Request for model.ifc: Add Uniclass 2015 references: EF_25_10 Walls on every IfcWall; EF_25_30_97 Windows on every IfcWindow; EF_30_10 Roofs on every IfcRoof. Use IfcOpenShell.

First a look at what the model holds.

```python
import ifcopenshell

model = ifcopenshell.open("model.ifc")
print(model.schema)
print("classifications:", [c.Name for c in model.by_type("IfcClassification")])
for ifc_class in ("IfcDoor", "IfcRoof", "IfcStair", "IfcWall", "IfcWindow"):
    print(ifc_class, len(model.by_type(ifc_class)))
```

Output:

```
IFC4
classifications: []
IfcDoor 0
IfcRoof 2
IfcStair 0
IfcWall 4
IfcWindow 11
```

```python
import ifcopenshell
import ifcopenshell.api.classification

model = ifcopenshell.open("model.ifc")

system = ifcopenshell.api.classification.add_classification(model, classification="Uniclass 2015")

codes = {
    "IfcWall": ("EF_25_10", "Walls"),
    "IfcWindow": ("EF_25_30_97", "Windows"),
    "IfcRoof": ("EF_30_10", "Roofs"),
}
for ifc_class, (code, name) in codes.items():
    products = model.by_type(ifc_class)
    ifcopenshell.api.classification.add_reference(
        model, products=products, classification=system, identification=code, name=name
    )
    print(code, len(products))

model.write("model-out.ifc")
```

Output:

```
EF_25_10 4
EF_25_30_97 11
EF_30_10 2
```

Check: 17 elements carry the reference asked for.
